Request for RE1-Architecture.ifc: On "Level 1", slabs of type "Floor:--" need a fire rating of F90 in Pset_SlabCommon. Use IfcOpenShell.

First a look at what the model holds.

```python
import ifcopenshell
import ifcopenshell.util.element

model = ifcopenshell.open("RE1-Architecture.ifc")
print(model.schema)
storey = next(s for s in model.by_type("IfcBuildingStorey") if s.Name == "Level 1")
slabs = [e for e in ifcopenshell.util.element.get_decomposition(storey) if e.is_a("IfcSlab")]
seen = {}
for e in slabs:
    element_type = ifcopenshell.util.element.get_type(e)
    key = (element_type.Name if element_type != e and element_type else None, ifcopenshell.util.element.get_pset(e, "Pset_SlabCommon", "FireRating"))
    seen[key] = seen.get(key, 0) + 1
for (name, value), count in sorted(seen.items(), key=str):
    print(count, "x", name, "|", value)
```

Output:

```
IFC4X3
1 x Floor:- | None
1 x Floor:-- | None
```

```python
import ifcopenshell
import ifcopenshell.api.pset
import ifcopenshell.util.element

model = ifcopenshell.open("RE1-Architecture.ifc")

storey = next(s for s in model.by_type("IfcBuildingStorey") if s.Name == "Level 1")
slabs = [e for e in ifcopenshell.util.element.get_decomposition(storey) if e.is_a("IfcSlab")]

count = 0
for e in slabs:
    element_type = ifcopenshell.util.element.get_type(e)
    if element_type in (None, e) or element_type.Name != "Floor:--":
        continue
    # add_pset returns the element's existing set when there is one.
    pset = ifcopenshell.api.pset.add_pset(model, product=e, name="Pset_SlabCommon")
    ifcopenshell.api.pset.edit_pset(model, pset=pset, properties={"FireRating": "F90"})
    count += 1

print(count, "slabs updated")

model.write("RE1-Architecture_rev.ifc")
```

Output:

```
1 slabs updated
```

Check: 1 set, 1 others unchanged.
